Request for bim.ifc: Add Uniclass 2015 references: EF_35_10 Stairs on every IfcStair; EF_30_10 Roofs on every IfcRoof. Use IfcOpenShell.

First a look at what the model holds.

```python
import ifcopenshell

model = ifcopenshell.open("bim.ifc")
print(model.schema)
print("classifications:", [c.Name for c in model.by_type("IfcClassification")])
for ifc_class in ("IfcDoor", "IfcRoof", "IfcStair", "IfcWall", "IfcWindow"):
    print(ifc_class, len(model.by_type(ifc_class)))
```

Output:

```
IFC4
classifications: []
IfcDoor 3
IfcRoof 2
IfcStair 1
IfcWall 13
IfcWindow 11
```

```python
import ifcopenshell
import ifcopenshell.api.classification

model = ifcopenshell.open("bim.ifc")

system = ifcopenshell.api.classification.add_classification(model, classification="Uniclass 2015")

codes = {
    "IfcStair": ("EF_35_10", "Stairs"),
    "IfcRoof": ("EF_30_10", "Roofs"),
}
for ifc_class, (code, name) in codes.items():
    products = model.by_type(ifc_class)
    ifcopenshell.api.classification.add_reference(
        model, products=products, classification=system, identification=code, name=name
    )
    print(code, len(products))

model.write("bim_v2.ifc")
```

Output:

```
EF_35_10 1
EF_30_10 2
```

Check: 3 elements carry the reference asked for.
